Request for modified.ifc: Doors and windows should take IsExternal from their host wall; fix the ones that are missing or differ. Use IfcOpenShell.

First a look at what the model holds.

```python
import ifcopenshell
import ifcopenshell.util.element

model = ifcopenshell.open("modified.ifc")
print(model.schema)
seen = {}
for e in model.by_type("IfcDoor") + model.by_type("IfcWindow"):
    if not e.FillsVoids:
        continue
    host = e.FillsVoids[0].RelatingOpeningElement.VoidsElements[0].RelatingBuildingElement
    own = ifcopenshell.util.element.get_pset(e, f"Pset_{e.is_a()[3:].removesuffix('StandardCase')}Common", "IsExternal")
    wall = ifcopenshell.util.element.get_pset(host, "Pset_WallCommon", "IsExternal")
    seen[e.is_a(), own, wall] = seen.get((e.is_a(), own, wall), 0) + 1
for (cls, own, wall), count in sorted(seen.items(), key=str):
    print(count, cls, "IsExternal:", own, "| host wall:", wall)
```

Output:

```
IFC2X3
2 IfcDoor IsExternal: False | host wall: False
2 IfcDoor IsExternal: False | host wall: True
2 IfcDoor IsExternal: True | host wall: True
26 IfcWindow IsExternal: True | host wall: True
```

```python
import ifcopenshell
import ifcopenshell.api.pset
import ifcopenshell.util.element

model = ifcopenshell.open("modified.ifc")

count = 0
for ifc_class, pset_name in (("IfcDoor", "Pset_DoorCommon"), ("IfcWindow", "Pset_WindowCommon")):
    for e in model.by_type(ifc_class):
        if not e.FillsVoids:
            continue
        host = e.FillsVoids[0].RelatingOpeningElement.VoidsElements[0].RelatingBuildingElement
        external = ifcopenshell.util.element.get_pset(host, "Pset_WallCommon", "IsExternal")
        if external is None or ifcopenshell.util.element.get_pset(e, pset_name, "IsExternal") == external:
            continue
        pset = ifcopenshell.api.pset.add_pset(model, product=e, name=pset_name)
        ifcopenshell.api.pset.edit_pset(model, pset=pset, properties={"IsExternal": external})
        count += 1

print(count, "updated")

model.write("modified_edited.ifc")
```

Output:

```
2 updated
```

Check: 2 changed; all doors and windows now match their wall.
